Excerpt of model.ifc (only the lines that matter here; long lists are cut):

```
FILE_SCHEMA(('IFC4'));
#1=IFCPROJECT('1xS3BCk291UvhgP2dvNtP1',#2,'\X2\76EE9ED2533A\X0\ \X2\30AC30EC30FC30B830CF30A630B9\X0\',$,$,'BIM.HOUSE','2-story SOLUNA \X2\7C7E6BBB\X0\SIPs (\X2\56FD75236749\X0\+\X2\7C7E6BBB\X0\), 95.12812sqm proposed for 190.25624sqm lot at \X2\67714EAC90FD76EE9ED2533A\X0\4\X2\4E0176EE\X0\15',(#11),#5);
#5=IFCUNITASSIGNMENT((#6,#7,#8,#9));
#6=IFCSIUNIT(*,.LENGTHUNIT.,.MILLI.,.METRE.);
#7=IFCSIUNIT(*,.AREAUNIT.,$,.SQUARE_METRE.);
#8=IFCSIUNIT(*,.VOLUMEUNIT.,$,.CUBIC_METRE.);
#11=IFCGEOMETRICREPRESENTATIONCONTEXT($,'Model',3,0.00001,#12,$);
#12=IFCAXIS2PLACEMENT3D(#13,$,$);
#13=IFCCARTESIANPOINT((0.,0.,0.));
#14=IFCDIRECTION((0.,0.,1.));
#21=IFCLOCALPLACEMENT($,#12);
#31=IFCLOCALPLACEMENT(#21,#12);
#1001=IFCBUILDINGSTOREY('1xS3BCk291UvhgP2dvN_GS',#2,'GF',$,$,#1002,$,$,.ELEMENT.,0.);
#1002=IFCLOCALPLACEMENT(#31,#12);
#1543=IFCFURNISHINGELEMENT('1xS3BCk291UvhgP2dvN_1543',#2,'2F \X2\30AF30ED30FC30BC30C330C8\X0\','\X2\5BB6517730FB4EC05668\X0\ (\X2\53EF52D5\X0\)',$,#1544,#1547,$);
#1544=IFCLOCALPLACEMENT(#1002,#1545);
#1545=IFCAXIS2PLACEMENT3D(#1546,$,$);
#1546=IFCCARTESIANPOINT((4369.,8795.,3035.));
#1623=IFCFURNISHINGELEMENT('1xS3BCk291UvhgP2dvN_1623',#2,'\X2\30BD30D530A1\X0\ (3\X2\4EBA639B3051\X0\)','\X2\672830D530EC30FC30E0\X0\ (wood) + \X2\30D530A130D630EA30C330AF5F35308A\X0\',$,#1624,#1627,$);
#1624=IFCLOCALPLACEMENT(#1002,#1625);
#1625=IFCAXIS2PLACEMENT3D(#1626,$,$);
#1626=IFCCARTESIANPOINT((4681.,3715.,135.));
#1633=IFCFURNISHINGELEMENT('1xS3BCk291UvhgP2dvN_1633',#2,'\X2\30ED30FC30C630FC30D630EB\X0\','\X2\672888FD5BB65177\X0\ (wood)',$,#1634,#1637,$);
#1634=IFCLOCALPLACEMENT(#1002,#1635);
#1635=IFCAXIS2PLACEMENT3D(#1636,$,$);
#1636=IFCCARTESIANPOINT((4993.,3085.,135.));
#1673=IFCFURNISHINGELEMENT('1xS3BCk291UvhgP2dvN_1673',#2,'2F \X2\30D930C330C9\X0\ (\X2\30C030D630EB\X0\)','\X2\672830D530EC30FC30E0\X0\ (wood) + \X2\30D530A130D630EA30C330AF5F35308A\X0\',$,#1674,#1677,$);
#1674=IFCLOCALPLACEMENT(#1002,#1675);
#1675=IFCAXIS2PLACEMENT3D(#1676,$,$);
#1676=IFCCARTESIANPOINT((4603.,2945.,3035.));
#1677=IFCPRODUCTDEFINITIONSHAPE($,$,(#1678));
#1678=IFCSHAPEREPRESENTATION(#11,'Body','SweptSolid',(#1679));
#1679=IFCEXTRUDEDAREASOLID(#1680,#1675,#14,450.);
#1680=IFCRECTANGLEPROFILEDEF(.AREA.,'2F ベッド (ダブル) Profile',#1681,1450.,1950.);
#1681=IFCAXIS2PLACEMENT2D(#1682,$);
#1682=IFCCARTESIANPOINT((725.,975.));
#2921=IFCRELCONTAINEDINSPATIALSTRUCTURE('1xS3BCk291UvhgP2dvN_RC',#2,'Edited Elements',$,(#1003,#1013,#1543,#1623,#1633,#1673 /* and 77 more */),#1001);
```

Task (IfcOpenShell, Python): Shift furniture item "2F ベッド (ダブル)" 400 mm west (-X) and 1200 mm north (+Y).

```python
import ifcopenshell
import ifcopenshell.api.geometry
import ifcopenshell.util.placement
import ifcopenshell.util.unit

model = ifcopenshell.open("model.ifc")
unit_scale = ifcopenshell.util.unit.calculate_unit_scale(model)

item = model.by_guid("1xS3BCk291UvhgP2dvN_1673")
matrix = ifcopenshell.util.placement.get_local_placement(item.ObjectPlacement)
matrix[0, 3] -= 0.4 / unit_scale
matrix[1, 3] += 1.2 / unit_scale
ifcopenshell.api.geometry.edit_object_placement(model, product=item, matrix=matrix, is_si=False)

print(ifcopenshell.util.placement.get_local_placement(item.ObjectPlacement).round(3) + 0.0)

model.write("model_rev.ifc")
```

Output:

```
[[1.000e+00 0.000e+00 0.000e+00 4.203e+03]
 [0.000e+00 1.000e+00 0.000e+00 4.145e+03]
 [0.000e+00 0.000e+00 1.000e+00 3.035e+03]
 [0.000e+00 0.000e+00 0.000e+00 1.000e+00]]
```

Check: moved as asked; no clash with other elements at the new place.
